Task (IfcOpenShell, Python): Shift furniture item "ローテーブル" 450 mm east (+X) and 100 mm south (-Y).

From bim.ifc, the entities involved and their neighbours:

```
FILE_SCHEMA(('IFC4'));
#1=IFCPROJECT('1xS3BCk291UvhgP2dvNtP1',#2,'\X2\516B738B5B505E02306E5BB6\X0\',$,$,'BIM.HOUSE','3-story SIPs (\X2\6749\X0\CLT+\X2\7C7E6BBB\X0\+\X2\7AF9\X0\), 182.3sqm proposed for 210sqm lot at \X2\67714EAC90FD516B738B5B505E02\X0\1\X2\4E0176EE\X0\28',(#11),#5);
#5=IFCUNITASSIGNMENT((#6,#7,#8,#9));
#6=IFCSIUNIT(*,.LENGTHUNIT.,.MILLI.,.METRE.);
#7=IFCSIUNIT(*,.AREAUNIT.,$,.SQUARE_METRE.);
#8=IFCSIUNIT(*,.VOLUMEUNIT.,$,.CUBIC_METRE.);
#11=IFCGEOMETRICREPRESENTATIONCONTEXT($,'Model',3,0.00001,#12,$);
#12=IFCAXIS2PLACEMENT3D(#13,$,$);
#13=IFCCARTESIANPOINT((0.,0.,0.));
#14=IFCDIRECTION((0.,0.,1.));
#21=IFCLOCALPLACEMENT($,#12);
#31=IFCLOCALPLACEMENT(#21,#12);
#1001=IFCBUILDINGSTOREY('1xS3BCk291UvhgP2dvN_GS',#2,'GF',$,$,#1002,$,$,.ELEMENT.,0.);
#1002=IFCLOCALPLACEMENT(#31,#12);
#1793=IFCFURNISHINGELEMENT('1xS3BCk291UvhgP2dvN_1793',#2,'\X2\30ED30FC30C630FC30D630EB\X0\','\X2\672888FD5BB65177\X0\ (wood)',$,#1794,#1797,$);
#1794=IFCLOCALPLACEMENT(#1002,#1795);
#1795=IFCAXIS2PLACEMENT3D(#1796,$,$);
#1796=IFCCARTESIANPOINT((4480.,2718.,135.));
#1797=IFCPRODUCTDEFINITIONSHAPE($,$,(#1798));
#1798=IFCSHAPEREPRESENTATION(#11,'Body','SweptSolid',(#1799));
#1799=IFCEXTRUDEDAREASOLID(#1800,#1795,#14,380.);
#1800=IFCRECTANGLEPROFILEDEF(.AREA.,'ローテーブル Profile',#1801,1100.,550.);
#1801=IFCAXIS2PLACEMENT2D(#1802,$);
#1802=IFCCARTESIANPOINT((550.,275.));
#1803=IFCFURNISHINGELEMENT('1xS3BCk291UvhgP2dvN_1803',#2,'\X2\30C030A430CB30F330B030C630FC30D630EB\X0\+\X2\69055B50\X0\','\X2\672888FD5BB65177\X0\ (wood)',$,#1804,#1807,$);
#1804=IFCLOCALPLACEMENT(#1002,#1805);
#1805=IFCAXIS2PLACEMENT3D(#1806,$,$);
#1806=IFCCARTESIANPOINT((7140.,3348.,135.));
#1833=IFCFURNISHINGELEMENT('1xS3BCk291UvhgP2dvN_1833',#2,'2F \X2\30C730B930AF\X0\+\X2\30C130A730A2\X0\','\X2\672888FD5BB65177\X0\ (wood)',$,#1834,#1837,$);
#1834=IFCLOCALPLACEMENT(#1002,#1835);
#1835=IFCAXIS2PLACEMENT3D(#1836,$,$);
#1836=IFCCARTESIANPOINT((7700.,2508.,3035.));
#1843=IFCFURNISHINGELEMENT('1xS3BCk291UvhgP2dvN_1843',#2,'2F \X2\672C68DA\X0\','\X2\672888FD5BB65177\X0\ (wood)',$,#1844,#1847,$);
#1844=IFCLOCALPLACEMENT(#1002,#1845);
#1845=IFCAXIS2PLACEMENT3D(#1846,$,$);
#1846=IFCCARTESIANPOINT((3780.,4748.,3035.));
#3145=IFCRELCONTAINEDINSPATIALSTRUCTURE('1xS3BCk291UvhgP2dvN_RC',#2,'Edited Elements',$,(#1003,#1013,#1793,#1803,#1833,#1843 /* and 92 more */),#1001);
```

```python
import ifcopenshell
import ifcopenshell.api.geometry
import ifcopenshell.util.placement
import ifcopenshell.util.unit

model = ifcopenshell.open("bim.ifc")
unit_scale = ifcopenshell.util.unit.calculate_unit_scale(model)

item = model.by_id(1793)
matrix = ifcopenshell.util.placement.get_local_placement(item.ObjectPlacement)
matrix[0, 3] += 0.45 / unit_scale
matrix[1, 3] -= 0.1 / unit_scale
ifcopenshell.api.geometry.edit_object_placement(model, product=item, matrix=matrix, is_si=False)

print(ifcopenshell.util.placement.get_local_placement(item.ObjectPlacement).round(3) + 0.0)

model.write("bim_edited.ifc")
```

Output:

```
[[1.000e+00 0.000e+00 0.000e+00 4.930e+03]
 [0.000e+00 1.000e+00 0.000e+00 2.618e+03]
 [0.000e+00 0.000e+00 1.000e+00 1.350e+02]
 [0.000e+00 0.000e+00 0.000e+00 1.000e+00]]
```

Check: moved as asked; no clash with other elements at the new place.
